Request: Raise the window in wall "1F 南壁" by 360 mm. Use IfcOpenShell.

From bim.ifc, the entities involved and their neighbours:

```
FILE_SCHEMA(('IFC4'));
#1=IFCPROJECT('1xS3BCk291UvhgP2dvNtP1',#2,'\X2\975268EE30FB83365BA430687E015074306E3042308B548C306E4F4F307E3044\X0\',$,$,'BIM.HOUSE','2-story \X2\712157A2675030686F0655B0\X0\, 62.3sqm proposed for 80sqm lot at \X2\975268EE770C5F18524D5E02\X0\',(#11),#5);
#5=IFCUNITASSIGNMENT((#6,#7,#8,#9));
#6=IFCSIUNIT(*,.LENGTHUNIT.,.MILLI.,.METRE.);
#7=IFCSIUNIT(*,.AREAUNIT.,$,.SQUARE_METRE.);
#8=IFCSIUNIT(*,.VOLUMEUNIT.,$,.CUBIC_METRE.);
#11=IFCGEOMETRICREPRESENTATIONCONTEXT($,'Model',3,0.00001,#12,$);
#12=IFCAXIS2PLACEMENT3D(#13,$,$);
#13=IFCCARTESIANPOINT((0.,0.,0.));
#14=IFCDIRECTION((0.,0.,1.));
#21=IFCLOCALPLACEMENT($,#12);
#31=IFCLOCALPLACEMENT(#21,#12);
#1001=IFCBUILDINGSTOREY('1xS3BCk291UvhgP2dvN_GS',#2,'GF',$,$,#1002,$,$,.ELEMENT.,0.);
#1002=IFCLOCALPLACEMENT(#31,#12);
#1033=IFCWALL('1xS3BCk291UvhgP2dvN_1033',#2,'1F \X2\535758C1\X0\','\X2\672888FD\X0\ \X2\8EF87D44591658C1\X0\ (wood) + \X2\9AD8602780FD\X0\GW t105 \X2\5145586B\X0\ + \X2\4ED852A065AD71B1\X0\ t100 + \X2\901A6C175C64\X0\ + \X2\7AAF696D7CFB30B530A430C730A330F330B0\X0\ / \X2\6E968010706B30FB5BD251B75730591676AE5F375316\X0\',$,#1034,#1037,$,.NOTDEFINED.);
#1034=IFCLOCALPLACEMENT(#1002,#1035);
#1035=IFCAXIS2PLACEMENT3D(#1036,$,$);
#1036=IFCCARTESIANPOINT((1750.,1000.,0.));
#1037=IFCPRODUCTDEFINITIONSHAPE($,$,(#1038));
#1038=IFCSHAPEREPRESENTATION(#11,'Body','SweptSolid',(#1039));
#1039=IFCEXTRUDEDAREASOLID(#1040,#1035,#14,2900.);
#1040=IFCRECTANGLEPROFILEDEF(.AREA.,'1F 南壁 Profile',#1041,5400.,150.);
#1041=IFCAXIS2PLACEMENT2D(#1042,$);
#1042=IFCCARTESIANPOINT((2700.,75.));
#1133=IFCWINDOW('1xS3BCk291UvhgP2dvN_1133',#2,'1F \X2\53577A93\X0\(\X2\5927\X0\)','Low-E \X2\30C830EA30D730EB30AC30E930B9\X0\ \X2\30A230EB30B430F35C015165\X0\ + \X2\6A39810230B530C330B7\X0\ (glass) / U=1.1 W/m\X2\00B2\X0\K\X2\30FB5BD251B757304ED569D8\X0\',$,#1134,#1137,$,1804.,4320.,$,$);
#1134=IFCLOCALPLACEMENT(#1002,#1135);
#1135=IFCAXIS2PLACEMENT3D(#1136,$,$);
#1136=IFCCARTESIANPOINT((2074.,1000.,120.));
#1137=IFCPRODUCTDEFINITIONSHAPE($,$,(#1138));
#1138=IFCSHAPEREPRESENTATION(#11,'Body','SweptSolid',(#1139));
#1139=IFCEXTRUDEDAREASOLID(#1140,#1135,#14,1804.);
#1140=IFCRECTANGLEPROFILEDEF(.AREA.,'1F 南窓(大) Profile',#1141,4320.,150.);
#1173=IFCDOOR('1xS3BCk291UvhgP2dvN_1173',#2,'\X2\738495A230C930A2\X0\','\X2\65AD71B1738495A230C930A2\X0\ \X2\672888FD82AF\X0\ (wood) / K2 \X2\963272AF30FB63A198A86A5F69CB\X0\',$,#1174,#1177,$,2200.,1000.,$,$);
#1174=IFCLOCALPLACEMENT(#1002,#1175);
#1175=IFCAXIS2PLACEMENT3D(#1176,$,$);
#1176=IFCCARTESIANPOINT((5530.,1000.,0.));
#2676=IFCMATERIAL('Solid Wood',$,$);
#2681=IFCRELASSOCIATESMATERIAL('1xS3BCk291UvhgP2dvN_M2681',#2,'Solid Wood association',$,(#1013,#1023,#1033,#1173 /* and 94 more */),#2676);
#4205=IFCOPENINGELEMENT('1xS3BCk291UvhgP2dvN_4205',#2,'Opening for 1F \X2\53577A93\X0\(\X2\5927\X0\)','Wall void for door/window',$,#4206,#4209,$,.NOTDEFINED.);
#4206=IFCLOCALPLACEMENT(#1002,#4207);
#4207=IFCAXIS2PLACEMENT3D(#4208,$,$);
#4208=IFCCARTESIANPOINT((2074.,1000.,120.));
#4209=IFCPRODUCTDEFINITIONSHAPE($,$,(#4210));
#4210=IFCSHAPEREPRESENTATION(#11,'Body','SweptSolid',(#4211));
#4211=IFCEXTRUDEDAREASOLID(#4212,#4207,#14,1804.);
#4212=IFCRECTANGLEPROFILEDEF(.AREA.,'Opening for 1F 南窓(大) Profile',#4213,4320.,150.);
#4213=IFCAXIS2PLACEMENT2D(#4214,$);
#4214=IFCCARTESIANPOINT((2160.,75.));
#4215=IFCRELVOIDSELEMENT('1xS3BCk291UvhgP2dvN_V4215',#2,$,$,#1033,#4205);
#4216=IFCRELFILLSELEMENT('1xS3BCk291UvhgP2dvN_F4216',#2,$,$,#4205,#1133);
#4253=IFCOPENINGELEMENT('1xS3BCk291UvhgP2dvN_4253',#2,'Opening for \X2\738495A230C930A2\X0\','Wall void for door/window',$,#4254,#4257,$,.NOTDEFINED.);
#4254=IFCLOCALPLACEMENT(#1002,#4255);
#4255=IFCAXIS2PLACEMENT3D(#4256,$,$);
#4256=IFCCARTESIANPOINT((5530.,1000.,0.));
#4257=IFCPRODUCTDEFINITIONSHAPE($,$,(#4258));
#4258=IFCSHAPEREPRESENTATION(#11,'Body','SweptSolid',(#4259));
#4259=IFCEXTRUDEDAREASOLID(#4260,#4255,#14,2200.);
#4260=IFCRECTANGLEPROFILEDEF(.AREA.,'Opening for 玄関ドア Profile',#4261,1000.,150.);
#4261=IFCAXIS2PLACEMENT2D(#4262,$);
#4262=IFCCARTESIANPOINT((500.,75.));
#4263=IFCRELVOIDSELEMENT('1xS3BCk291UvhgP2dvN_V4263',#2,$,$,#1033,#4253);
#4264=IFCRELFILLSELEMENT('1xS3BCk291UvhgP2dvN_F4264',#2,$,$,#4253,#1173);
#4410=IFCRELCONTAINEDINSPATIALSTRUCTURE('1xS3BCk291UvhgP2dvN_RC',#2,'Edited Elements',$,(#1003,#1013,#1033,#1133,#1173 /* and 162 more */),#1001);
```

```python
import numpy as np
import ifcopenshell
import ifcopenshell.api.geometry
import ifcopenshell.util.placement
import ifcopenshell.util.unit

model = ifcopenshell.open("bim.ifc")
unit_scale = ifcopenshell.util.unit.calculate_unit_scale(model)

window = model.by_id(1133)
opening = window.FillsVoids[0].RelatingOpeningElement
dz = 360.0

shift = np.array([0.0, 0.0, dz])
# The window is not placed relative to its opening, so move both.
for product in (opening, window):
    matrix = ifcopenshell.util.placement.get_local_placement(product.ObjectPlacement)
    matrix[:3, 3] += shift
    ifcopenshell.api.geometry.edit_object_placement(model, product=product, matrix=matrix, is_si=False)

print(f"moved by {dz * unit_scale:+.3f} m")

model.write("bim_updated.ifc")
```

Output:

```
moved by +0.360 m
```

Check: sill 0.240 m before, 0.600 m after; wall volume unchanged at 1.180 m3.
